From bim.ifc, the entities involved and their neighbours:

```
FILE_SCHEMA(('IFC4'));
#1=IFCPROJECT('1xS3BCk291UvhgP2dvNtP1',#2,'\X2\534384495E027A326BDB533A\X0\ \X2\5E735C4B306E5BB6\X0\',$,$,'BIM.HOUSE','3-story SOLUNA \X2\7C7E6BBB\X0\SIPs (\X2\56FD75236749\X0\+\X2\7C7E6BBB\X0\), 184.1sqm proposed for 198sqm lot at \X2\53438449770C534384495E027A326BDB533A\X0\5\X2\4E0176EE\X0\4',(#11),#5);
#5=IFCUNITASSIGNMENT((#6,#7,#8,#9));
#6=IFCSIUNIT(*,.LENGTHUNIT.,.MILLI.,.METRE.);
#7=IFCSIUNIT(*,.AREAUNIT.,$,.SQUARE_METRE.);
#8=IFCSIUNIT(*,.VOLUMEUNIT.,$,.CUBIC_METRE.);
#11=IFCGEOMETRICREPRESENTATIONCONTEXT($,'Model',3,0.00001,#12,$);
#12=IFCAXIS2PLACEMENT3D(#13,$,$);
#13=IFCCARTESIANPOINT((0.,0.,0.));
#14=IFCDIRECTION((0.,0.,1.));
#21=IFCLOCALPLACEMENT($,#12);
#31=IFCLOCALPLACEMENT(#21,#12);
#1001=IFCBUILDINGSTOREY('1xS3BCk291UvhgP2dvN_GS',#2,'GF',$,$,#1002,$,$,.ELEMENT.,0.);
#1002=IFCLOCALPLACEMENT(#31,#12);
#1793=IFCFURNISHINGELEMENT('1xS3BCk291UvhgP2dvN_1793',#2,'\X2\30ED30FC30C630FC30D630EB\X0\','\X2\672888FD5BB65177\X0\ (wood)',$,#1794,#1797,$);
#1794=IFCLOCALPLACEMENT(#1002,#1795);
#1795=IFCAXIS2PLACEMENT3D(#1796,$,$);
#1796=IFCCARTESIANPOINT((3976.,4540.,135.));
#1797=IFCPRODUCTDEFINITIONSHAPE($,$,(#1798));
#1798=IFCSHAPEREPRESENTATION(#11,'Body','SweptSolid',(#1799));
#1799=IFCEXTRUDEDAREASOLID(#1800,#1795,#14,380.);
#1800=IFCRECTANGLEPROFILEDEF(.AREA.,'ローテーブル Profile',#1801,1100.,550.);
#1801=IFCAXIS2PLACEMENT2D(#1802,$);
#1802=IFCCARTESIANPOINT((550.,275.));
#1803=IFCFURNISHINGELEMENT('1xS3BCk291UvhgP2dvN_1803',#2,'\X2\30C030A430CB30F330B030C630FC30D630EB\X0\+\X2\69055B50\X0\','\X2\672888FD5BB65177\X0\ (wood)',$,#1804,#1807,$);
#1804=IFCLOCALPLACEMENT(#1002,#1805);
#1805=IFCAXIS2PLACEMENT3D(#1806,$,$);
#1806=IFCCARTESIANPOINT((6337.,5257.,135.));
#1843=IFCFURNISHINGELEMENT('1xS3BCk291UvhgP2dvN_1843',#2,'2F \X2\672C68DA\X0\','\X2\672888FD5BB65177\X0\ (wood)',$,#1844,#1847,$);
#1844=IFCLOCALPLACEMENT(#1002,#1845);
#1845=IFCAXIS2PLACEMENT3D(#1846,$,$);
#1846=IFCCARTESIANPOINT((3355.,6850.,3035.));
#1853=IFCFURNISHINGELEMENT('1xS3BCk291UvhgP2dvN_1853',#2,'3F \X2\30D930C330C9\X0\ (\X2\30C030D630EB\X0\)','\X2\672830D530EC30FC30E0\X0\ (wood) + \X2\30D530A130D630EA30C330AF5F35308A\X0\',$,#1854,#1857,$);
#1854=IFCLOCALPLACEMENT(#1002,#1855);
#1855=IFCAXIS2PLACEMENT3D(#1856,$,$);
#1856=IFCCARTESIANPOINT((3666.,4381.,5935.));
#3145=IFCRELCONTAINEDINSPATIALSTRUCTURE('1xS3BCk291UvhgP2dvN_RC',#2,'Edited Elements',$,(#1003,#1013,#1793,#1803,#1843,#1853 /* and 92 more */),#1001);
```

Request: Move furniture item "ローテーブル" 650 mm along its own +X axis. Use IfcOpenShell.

```python
import ifcopenshell
import ifcopenshell.api.geometry
import ifcopenshell.util.placement
import ifcopenshell.util.unit

model = ifcopenshell.open("bim.ifc")
unit_scale = ifcopenshell.util.unit.calculate_unit_scale(model)

item = model.by_id(1793)
matrix = ifcopenshell.util.placement.get_local_placement(item.ObjectPlacement)
matrix[:3, 3] += matrix[:3, 0] * 0.65 / unit_scale
ifcopenshell.api.geometry.edit_object_placement(model, product=item, matrix=matrix, is_si=False)

print(ifcopenshell.util.placement.get_local_placement(item.ObjectPlacement).round(3) + 0.0)

model.write("bim_updated.ifc")
```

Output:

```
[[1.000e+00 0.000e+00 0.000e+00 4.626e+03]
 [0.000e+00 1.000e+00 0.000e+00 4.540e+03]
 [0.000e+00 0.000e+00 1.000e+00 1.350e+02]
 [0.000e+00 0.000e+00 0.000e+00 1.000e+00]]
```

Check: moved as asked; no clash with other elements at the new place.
